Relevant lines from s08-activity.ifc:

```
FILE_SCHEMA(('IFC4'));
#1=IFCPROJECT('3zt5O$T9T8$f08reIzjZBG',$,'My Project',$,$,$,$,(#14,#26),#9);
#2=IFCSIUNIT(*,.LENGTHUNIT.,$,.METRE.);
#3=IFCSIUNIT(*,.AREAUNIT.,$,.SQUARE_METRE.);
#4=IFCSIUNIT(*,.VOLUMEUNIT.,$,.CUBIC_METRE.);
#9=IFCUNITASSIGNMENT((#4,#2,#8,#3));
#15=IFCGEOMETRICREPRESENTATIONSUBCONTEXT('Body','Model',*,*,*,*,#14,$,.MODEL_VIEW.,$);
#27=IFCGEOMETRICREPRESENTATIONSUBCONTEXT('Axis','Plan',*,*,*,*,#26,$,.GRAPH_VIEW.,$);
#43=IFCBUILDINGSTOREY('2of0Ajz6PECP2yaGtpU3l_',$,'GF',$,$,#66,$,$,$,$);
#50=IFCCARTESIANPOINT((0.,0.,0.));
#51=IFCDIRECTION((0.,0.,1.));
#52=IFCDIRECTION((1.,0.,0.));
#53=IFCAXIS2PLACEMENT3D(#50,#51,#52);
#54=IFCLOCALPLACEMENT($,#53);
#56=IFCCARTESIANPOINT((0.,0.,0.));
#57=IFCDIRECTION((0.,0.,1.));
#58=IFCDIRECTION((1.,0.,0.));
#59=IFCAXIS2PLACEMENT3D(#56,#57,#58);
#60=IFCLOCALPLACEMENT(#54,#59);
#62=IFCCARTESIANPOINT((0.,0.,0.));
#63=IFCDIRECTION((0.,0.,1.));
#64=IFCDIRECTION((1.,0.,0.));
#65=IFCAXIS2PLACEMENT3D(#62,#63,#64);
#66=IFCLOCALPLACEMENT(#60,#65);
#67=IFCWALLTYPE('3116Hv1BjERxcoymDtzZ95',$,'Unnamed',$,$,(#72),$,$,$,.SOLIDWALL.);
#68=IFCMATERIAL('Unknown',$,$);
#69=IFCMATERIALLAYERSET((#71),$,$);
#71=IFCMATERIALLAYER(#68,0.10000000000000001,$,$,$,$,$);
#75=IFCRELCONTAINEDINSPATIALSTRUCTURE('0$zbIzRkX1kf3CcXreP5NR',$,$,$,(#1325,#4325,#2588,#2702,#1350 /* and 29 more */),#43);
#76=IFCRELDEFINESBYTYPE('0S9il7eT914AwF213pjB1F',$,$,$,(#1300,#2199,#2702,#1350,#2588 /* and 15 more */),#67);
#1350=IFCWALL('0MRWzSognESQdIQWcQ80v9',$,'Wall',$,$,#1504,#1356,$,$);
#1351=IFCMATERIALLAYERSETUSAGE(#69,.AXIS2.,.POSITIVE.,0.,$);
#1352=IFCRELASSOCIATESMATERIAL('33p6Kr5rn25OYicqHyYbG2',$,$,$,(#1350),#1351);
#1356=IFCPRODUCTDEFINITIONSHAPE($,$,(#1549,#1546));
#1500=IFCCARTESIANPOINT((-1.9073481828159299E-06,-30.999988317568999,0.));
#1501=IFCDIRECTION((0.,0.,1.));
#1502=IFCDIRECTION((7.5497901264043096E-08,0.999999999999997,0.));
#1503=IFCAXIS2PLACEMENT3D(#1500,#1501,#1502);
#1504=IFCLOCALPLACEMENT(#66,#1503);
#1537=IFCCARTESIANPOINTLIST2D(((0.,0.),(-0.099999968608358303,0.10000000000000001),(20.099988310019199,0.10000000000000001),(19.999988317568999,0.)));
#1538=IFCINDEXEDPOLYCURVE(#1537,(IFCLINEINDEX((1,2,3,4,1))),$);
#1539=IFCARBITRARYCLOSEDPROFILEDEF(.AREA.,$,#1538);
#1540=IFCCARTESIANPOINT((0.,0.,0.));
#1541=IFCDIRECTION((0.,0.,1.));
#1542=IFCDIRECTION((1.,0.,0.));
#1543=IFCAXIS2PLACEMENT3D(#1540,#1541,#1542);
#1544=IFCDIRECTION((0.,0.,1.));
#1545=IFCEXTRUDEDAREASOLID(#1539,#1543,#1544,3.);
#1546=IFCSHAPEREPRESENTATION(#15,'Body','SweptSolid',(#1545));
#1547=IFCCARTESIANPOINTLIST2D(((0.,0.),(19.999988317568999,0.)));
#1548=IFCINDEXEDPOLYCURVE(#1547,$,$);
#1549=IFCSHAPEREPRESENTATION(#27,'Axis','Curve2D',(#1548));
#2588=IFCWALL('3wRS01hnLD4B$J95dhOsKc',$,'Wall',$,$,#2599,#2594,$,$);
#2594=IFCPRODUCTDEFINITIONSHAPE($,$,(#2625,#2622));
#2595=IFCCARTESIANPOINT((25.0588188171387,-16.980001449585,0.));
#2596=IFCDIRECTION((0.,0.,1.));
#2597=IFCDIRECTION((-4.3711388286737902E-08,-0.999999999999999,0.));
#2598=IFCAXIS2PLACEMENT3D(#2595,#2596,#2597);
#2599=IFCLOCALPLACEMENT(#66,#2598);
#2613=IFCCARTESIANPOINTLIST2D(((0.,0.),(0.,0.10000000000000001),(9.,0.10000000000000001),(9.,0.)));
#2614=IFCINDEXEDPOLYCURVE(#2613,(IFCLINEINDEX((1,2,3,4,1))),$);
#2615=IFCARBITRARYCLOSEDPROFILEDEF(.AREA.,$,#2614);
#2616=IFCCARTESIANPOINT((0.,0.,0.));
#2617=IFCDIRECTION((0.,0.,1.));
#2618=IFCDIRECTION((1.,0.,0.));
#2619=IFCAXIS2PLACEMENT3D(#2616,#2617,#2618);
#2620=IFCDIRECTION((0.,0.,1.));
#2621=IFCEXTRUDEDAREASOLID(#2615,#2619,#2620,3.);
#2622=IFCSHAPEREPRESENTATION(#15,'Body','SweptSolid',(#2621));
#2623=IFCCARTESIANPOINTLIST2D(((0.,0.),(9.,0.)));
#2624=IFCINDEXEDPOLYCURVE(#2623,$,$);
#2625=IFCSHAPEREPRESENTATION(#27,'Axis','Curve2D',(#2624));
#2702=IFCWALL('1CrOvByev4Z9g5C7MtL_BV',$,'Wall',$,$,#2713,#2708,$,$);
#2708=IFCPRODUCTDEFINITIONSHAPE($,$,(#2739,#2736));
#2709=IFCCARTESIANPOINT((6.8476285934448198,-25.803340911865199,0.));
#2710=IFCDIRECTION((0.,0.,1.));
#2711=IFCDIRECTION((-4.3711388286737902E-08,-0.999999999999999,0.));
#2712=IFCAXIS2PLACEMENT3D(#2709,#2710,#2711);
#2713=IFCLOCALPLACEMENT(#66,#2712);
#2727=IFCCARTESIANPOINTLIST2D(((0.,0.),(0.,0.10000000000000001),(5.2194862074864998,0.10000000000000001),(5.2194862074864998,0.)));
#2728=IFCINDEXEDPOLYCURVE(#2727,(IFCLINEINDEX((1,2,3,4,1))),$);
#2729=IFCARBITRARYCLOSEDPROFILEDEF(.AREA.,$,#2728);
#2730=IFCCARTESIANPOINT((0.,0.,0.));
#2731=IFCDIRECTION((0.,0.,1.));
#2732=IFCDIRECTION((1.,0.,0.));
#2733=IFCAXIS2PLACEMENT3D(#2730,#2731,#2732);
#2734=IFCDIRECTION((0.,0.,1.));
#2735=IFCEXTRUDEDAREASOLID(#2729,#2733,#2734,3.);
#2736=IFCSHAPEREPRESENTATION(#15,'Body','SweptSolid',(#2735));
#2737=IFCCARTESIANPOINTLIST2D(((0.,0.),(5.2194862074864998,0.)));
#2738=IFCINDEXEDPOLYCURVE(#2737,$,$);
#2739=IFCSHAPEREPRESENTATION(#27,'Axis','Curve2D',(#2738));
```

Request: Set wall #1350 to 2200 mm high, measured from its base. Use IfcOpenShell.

```python
import ifcopenshell
import ifcopenshell.geom
import ifcopenshell.util.representation
import ifcopenshell.util.shape
import ifcopenshell.util.unit

model = ifcopenshell.open("s08-activity.ifc")
unit_scale = ifcopenshell.util.unit.calculate_unit_scale(model)
settings = ifcopenshell.geom.settings()


def volume(element):
    """Net volume in cubic metres, openings subtracted."""
    shape = ifcopenshell.geom.create_shape(settings, element)
    return ifcopenshell.util.shape.get_volume(shape.geometry)


wall = model.by_guid("0MRWzSognESQdIQWcQ80v9")
before = volume(wall)

body = ifcopenshell.util.representation.get_representation(wall, "Model", "Body")
solid = body.Items[0]
old_height = solid.Depth
solid.Depth = 2.2 / unit_scale
after = volume(wall)

print(f"height {old_height:g} -> {solid.Depth:g}, volume {before:.3f} -> {after:.3f} m3")

model.write("s08-activity_updated.ifc")
```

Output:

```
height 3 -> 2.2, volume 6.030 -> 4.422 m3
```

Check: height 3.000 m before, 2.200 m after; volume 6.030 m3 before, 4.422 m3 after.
